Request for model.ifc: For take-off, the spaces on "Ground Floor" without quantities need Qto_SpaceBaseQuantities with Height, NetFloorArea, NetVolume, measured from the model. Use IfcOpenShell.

First a look at what the model holds.

```python
import ifcopenshell
import ifcopenshell.util.element
import ifcopenshell.util.unit

model = ifcopenshell.open("model.ifc")
print(model.schema)
for unit_type in ("LENGTHUNIT", "AREAUNIT", "VOLUMEUNIT"):
    print(unit_type, ifcopenshell.util.unit.calculate_unit_scale(model, unit_type))
storey = next(s for s in model.by_type("IfcBuildingStorey") if s.Name == "Ground Floor")
spaces = [e for e in ifcopenshell.util.element.get_decomposition(storey) if e.is_a("IfcSpace")]
for e in sorted(spaces, key=lambda e: e.id()):
    print(e.id(), e.is_a(), e.Name, list(ifcopenshell.util.element.get_psets(e, qtos_only=True)), sep=" | ")
```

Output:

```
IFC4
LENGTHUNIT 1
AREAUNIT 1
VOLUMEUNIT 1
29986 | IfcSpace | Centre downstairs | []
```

```python
import ifcopenshell
import ifcopenshell.api.pset
import ifcopenshell.geom
import ifcopenshell.util.element
import ifcopenshell.util.shape
import ifcopenshell.util.unit

model = ifcopenshell.open("model.ifc")
unit_scale = ifcopenshell.util.unit.calculate_unit_scale(model)
area_scale = ifcopenshell.util.unit.calculate_unit_scale(model, "AREAUNIT")
volume_scale = ifcopenshell.util.unit.calculate_unit_scale(model, "VOLUMEUNIT")
settings = ifcopenshell.geom.settings()

storey = next(s for s in model.by_type("IfcBuildingStorey") if s.Name == "Ground Floor")
spaces = [e for e in ifcopenshell.util.element.get_decomposition(storey) if e.is_a("IfcSpace")]

for e in sorted(spaces, key=lambda e: e.id()):
    if ifcopenshell.util.element.get_psets(e, qtos_only=True, should_inherit=False):
        continue
    # Geometry comes back in metres, in the element's own axes.
    shape = ifcopenshell.geom.create_shape(settings, e)
    values = {
        "Height": ifcopenshell.util.shape.get_z(shape.geometry) / unit_scale,
        "NetFloorArea": ifcopenshell.util.shape.get_footprint_area(shape.geometry) / area_scale,
        "NetVolume": ifcopenshell.util.shape.get_volume(shape.geometry) / volume_scale,
    }
    qto = ifcopenshell.api.pset.add_qto(model, product=e, name="Qto_SpaceBaseQuantities")
    ifcopenshell.api.pset.edit_qto(model, qto=qto, properties=values)
    print(e.id(), {k: round(v, 3) for k, v in values.items()})

model.write("model_rev.ifc")
```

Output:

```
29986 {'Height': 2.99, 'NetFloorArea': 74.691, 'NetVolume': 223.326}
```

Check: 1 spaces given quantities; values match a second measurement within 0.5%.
